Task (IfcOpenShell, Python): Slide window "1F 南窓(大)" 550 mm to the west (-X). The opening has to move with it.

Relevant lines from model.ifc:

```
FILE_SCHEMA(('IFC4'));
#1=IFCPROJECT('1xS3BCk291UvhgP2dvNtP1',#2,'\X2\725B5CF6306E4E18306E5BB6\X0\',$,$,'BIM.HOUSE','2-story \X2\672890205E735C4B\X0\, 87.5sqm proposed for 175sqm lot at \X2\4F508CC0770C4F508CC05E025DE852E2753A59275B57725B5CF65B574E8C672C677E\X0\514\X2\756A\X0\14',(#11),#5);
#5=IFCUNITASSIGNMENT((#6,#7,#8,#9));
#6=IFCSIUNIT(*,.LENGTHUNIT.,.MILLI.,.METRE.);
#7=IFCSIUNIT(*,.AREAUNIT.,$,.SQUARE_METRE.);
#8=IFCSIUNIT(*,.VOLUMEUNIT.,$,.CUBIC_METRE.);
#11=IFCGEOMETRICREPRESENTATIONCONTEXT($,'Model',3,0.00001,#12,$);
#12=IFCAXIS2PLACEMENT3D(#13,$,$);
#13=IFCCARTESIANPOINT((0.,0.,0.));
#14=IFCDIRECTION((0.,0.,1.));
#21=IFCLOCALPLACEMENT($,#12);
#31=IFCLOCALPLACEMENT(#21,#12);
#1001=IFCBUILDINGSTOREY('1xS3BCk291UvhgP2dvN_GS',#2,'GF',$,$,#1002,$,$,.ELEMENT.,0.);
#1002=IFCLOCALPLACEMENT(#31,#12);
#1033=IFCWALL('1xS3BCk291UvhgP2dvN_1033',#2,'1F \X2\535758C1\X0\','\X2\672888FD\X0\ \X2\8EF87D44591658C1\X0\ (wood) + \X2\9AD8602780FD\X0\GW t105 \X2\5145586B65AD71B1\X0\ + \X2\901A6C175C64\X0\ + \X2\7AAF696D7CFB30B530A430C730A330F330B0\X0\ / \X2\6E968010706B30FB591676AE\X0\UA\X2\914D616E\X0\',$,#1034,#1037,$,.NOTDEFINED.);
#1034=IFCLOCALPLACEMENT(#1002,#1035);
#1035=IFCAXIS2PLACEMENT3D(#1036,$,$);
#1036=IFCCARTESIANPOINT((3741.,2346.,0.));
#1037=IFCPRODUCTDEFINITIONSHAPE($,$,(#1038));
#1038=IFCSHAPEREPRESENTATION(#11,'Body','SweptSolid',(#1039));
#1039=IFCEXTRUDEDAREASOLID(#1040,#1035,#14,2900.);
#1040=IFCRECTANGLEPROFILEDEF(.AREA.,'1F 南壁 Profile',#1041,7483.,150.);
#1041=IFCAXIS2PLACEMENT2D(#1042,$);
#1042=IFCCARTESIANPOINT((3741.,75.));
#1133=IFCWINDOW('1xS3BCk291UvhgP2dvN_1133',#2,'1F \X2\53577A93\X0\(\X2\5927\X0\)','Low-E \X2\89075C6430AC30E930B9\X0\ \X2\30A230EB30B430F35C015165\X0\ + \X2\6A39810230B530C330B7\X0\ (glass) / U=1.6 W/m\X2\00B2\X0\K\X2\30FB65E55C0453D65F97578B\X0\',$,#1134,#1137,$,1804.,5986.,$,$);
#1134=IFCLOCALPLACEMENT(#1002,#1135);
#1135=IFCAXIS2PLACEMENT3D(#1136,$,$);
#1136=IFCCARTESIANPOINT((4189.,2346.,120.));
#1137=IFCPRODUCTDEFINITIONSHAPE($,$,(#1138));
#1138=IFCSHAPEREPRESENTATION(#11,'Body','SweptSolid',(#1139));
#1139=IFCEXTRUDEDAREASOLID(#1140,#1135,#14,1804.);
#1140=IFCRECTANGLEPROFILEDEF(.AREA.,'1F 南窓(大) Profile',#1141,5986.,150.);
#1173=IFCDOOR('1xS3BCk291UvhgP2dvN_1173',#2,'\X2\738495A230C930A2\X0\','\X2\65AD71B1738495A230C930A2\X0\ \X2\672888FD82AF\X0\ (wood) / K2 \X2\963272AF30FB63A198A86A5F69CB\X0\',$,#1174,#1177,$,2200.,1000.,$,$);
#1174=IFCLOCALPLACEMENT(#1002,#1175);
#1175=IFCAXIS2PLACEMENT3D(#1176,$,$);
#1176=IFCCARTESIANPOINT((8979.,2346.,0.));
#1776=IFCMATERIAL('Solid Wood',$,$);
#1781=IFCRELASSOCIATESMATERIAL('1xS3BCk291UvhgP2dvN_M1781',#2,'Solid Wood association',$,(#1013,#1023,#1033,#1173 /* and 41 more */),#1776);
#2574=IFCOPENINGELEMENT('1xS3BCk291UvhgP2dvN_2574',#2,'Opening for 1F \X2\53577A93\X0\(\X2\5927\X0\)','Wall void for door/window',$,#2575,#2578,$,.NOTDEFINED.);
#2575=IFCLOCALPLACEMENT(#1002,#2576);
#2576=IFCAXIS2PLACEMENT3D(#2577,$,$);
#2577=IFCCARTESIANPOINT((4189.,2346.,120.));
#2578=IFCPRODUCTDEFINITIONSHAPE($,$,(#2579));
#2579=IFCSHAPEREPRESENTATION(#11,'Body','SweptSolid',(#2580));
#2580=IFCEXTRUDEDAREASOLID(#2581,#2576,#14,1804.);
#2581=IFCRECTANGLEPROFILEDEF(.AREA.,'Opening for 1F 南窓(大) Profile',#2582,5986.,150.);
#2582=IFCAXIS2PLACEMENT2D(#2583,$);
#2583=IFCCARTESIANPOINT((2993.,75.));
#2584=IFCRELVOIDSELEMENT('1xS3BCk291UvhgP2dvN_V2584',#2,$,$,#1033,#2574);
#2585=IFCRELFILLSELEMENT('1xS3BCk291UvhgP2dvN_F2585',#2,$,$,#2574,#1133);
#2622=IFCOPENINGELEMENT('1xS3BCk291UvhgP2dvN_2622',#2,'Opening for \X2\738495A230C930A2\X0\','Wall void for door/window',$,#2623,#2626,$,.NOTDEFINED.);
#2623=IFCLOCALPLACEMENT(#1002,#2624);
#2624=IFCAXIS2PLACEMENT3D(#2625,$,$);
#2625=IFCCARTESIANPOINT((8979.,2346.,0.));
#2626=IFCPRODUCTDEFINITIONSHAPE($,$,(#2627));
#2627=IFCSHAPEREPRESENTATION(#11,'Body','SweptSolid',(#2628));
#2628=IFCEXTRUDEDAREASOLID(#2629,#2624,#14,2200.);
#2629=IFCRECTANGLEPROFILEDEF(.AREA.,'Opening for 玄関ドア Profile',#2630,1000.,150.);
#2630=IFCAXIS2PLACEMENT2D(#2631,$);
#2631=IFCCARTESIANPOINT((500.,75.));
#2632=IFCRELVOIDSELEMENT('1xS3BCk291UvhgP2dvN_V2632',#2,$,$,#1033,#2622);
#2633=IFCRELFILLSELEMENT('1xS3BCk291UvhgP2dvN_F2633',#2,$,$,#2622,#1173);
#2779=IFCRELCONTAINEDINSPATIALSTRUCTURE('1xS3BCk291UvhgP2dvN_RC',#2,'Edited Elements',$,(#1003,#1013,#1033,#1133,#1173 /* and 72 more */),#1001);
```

```python
import ifcopenshell
import ifcopenshell.api.geometry
import ifcopenshell.util.placement
import ifcopenshell.util.unit

model = ifcopenshell.open("model.ifc")
unit_scale = ifcopenshell.util.unit.calculate_unit_scale(model)

window = model.by_id(1133)
opening = window.FillsVoids[0].RelatingOpeningElement
wall = opening.VoidsElements[0].RelatingBuildingElement

wall_matrix = ifcopenshell.util.placement.get_local_placement(wall.ObjectPlacement)
shift = wall_matrix[:3, 0] * -0.55 / unit_scale
before = ifcopenshell.util.placement.get_local_placement(window.ObjectPlacement)[:3, 3].copy()

# The window is not placed relative to its opening, so move both.
for product in (opening, window):
    matrix = ifcopenshell.util.placement.get_local_placement(product.ObjectPlacement)
    matrix[:3, 3] += shift
    ifcopenshell.api.geometry.edit_object_placement(model, product=product, matrix=matrix, is_si=False)

after = ifcopenshell.util.placement.get_local_placement(window.ObjectPlacement)[:3, 3]
print("window moved by", (after - before).round(3) + 0.0)

model.write("model-out.ifc")
```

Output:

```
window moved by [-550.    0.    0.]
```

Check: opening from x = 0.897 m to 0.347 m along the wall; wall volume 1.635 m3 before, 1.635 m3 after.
